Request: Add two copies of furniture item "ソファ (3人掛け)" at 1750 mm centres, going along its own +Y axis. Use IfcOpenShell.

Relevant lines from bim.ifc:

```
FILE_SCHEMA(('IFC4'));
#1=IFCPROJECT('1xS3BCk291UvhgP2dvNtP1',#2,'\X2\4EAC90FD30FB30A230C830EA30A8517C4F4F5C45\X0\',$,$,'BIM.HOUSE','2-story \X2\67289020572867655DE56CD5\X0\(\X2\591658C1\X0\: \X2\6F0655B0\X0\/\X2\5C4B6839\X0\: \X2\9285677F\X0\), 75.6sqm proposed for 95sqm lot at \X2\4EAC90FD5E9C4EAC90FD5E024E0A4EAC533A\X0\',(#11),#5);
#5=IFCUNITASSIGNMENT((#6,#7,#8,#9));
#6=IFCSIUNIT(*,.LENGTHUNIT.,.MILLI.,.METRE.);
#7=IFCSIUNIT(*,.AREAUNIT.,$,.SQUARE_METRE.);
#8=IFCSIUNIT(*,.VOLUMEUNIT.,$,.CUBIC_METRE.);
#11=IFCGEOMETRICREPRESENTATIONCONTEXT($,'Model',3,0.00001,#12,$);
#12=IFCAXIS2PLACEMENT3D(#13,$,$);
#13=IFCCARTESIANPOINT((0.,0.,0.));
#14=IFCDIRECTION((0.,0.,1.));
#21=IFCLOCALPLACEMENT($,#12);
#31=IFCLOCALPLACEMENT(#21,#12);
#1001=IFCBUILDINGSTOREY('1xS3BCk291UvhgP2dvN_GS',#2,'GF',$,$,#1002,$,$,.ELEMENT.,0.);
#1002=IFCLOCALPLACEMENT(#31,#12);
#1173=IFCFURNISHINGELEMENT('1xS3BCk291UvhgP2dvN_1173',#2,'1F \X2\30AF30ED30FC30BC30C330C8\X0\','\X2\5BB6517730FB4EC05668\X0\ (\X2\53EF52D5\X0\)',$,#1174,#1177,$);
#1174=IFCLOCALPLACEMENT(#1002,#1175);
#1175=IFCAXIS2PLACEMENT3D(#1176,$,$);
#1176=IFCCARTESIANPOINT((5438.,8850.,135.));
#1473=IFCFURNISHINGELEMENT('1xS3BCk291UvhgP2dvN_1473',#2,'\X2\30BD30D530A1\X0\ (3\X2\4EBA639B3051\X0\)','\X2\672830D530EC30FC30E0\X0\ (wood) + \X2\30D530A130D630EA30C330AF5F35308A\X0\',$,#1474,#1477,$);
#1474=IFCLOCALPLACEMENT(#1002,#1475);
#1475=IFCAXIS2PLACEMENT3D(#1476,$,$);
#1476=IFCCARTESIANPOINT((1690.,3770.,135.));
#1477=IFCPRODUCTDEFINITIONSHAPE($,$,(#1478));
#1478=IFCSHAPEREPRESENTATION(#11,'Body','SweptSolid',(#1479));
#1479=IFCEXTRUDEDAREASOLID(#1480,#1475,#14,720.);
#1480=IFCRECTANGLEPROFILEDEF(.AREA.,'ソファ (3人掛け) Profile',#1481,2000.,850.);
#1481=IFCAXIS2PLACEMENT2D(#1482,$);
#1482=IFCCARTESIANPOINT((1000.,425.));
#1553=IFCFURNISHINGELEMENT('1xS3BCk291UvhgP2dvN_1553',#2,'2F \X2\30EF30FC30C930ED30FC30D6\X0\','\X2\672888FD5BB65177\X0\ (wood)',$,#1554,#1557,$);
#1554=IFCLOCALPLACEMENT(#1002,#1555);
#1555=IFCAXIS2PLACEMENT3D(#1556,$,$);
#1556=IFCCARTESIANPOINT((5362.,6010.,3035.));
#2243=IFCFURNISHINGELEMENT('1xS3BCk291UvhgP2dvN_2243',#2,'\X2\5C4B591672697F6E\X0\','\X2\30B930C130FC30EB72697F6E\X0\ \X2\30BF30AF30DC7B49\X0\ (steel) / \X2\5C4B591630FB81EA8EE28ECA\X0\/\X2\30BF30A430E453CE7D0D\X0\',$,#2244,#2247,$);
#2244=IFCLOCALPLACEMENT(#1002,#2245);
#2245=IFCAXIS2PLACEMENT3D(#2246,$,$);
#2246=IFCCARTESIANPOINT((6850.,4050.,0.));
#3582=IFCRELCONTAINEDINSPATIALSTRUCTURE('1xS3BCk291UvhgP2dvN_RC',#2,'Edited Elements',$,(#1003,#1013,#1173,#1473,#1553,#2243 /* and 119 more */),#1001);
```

```python
import ifcopenshell
import ifcopenshell.api.geometry
import ifcopenshell.api.root
import ifcopenshell.util.element
import ifcopenshell.util.placement
import ifcopenshell.util.unit

model = ifcopenshell.open("bim.ifc")
unit_scale = ifcopenshell.util.unit.calculate_unit_scale(model)


def reuse_history(source, copy):
    """copy_class also copies each property set's owner history, people and application; keep the originals."""
    for rel in copy.IsDefinedBy:
        if rel.is_a("IfcRelDefinesByProperties") and (history := rel.RelatingPropertyDefinition.OwnerHistory):
            rel.RelatingPropertyDefinition.OwnerHistory = source.OwnerHistory
            ifcopenshell.util.element.remove_deep2(model, history)


source = model.by_id(1473)
base = ifcopenshell.util.placement.get_local_placement(source.ObjectPlacement)
step = base[:3, 1] * 1.75 / unit_scale

for i in range(1, 3):
    copy = ifcopenshell.api.root.copy_class(model, product=source)
    copy.Representation = ifcopenshell.util.element.copy_deep(
        model, source.Representation, exclude=["IfcGeometricRepresentationContext", "IfcRepresentationMap"]
    )
    reuse_history(source, copy)
    matrix = base.copy()
    matrix[:3, 3] += i * step
    print("added at", matrix[:3, 3].round(3) + 0.0)
    ifcopenshell.api.geometry.edit_object_placement(model, product=copy, matrix=matrix, is_si=False)

model.write("bim_updated.ifc")
```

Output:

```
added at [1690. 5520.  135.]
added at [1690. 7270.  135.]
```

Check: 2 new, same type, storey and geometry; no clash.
